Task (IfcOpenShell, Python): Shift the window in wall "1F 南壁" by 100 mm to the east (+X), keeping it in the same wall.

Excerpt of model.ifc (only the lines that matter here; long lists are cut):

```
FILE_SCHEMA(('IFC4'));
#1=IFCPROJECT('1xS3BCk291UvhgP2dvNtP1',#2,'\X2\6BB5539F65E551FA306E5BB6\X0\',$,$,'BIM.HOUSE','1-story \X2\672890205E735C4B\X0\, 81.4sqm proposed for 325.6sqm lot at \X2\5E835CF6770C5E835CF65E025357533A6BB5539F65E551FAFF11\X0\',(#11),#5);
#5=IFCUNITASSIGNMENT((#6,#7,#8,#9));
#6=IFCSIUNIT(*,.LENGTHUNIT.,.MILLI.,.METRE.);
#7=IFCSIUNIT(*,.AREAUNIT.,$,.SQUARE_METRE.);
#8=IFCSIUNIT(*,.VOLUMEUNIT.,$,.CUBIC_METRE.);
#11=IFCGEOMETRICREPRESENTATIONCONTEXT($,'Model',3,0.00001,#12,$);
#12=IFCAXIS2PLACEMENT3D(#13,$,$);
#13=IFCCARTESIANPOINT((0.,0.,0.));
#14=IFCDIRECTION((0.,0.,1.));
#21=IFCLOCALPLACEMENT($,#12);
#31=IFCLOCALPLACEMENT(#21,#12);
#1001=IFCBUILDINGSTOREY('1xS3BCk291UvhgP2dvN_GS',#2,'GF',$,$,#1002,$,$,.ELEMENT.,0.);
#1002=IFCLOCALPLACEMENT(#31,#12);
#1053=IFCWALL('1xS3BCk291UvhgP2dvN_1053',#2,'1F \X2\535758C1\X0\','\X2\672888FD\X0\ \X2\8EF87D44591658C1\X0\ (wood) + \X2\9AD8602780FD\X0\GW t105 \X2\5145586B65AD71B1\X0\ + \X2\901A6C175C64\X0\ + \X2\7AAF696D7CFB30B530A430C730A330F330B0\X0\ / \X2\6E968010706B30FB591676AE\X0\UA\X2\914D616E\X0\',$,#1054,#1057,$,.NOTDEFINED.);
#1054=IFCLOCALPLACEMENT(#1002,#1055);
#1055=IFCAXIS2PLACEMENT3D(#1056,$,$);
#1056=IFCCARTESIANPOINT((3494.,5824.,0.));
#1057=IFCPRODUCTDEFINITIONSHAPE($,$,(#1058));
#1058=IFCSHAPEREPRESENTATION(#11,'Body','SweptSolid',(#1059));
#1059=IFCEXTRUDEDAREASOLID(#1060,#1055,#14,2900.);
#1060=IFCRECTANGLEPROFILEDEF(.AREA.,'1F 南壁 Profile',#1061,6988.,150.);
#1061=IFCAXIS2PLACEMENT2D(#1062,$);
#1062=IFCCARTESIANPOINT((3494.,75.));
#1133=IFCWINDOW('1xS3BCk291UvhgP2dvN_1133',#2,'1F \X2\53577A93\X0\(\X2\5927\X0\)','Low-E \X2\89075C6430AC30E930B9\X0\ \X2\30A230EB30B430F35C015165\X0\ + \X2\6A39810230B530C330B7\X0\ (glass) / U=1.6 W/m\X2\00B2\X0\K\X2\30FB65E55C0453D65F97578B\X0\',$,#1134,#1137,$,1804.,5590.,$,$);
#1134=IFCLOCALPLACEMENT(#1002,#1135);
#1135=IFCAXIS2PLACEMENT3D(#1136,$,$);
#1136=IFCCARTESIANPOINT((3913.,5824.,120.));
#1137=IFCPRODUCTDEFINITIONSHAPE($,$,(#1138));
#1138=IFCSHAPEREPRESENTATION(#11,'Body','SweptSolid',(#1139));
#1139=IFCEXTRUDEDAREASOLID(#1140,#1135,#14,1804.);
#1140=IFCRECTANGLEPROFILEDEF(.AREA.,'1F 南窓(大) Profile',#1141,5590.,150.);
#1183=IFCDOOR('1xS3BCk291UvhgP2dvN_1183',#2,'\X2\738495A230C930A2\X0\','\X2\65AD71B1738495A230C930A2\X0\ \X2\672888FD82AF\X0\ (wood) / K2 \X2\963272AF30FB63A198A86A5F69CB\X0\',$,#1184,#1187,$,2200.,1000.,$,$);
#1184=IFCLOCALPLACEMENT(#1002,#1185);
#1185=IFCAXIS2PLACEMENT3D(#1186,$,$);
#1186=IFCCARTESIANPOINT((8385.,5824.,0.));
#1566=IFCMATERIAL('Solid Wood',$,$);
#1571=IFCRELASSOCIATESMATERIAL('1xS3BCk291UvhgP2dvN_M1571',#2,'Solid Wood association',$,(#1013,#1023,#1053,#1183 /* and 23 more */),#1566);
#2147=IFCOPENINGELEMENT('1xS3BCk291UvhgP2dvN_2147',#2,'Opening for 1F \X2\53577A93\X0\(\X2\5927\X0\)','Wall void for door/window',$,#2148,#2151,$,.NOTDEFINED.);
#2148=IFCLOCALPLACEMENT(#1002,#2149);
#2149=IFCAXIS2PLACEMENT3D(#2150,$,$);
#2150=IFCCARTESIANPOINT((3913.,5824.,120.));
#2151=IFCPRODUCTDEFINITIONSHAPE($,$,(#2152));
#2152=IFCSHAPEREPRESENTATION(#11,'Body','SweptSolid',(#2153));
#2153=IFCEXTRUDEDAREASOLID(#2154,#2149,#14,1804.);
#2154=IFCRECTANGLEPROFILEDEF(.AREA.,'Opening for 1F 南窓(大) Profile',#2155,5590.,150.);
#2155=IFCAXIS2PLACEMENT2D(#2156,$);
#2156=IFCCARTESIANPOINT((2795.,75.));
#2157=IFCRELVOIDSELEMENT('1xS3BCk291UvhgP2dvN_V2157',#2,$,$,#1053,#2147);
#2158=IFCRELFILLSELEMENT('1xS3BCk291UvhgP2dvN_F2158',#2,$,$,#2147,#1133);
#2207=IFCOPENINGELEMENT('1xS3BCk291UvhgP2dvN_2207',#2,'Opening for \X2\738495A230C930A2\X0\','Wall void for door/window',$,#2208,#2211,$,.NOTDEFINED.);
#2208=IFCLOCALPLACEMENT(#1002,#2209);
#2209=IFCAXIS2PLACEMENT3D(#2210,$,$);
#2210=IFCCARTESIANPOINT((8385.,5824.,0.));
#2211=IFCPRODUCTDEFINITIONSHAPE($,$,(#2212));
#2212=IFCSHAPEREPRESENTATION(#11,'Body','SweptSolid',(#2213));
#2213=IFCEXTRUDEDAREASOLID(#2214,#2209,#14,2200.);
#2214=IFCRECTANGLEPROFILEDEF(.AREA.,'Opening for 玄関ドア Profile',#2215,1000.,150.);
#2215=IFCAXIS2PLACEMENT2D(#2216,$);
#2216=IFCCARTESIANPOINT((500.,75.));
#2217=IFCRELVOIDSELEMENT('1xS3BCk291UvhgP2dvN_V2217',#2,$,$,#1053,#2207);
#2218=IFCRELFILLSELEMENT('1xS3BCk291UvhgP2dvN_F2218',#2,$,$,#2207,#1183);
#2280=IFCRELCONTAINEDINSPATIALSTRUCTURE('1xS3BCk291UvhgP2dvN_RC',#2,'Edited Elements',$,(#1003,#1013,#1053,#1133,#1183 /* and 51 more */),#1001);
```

```python
import ifcopenshell
import ifcopenshell.api.geometry
import ifcopenshell.util.placement
import ifcopenshell.util.unit

model = ifcopenshell.open("model.ifc")
unit_scale = ifcopenshell.util.unit.calculate_unit_scale(model)

window = model.by_guid("1xS3BCk291UvhgP2dvN_1133")
opening = window.FillsVoids[0].RelatingOpeningElement
wall = opening.VoidsElements[0].RelatingBuildingElement

wall_matrix = ifcopenshell.util.placement.get_local_placement(wall.ObjectPlacement)
shift = wall_matrix[:3, 0] * 0.1 / unit_scale
before = ifcopenshell.util.placement.get_local_placement(window.ObjectPlacement)[:3, 3].copy()

# The window is not placed relative to its opening, so move both.
for product in (opening, window):
    matrix = ifcopenshell.util.placement.get_local_placement(product.ObjectPlacement)
    matrix[:3, 3] += shift
    ifcopenshell.api.geometry.edit_object_placement(model, product=product, matrix=matrix, is_si=False)

after = ifcopenshell.util.placement.get_local_placement(window.ObjectPlacement)[:3, 3]
print("window moved by", (after - before).round(3) + 0.0)

model.write("model_v2.ifc")
```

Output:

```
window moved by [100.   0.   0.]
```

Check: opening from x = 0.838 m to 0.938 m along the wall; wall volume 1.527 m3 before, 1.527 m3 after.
